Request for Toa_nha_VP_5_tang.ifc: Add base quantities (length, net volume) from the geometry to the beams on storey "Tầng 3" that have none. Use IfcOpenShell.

First a look at what the model holds.

```python
import ifcopenshell
import ifcopenshell.util.element
import ifcopenshell.util.unit

model = ifcopenshell.open("Toa_nha_VP_5_tang.ifc")
print(model.schema)
for unit_type in ("LENGTHUNIT", "AREAUNIT", "VOLUMEUNIT"):
    print(unit_type, ifcopenshell.util.unit.calculate_unit_scale(model, unit_type))
storey = next(s for s in model.by_type("IfcBuildingStorey") if s.Name == "Tầng 3")
beams = [e for e in ifcopenshell.util.element.get_decomposition(storey) if e.is_a("IfcBeam")]
for e in sorted(beams, key=lambda e: e.id()):
    print(e.id(), e.is_a(), e.Name, list(ifcopenshell.util.element.get_psets(e, qtos_only=True)), sep=" | ")
```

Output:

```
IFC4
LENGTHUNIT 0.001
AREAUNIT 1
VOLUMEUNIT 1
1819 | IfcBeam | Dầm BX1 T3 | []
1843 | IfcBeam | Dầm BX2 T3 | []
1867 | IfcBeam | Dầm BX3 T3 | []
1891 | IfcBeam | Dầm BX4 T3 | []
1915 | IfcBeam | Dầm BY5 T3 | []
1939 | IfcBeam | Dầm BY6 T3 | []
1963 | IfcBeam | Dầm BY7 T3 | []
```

```python
import ifcopenshell
import ifcopenshell.api.pset
import ifcopenshell.geom
import ifcopenshell.util.element
import ifcopenshell.util.shape
import ifcopenshell.util.unit

model = ifcopenshell.open("Toa_nha_VP_5_tang.ifc")
unit_scale = ifcopenshell.util.unit.calculate_unit_scale(model)
volume_scale = ifcopenshell.util.unit.calculate_unit_scale(model, "VOLUMEUNIT")
settings = ifcopenshell.geom.settings()

storey = next(s for s in model.by_type("IfcBuildingStorey") if s.Name == "Tầng 3")
beams = [e for e in ifcopenshell.util.element.get_decomposition(storey) if e.is_a("IfcBeam")]

for e in sorted(beams, key=lambda e: e.id()):
    if ifcopenshell.util.element.get_psets(e, qtos_only=True, should_inherit=False):
        continue
    # Geometry comes back in metres, in the element's own axes.
    shape = ifcopenshell.geom.create_shape(settings, e)
    values = {
        "Length": ifcopenshell.util.shape.get_max_xyz(shape.geometry) / unit_scale,
        "NetVolume": ifcopenshell.util.shape.get_volume(shape.geometry) / volume_scale,
    }
    qto = ifcopenshell.api.pset.add_qto(model, product=e, name="Qto_BeamBaseQuantities")
    ifcopenshell.api.pset.edit_qto(model, qto=qto, properties=values)
    print(e.id(), {k: round(v, 3) for k, v in values.items()})

model.write("Toa_nha_VP_5_tang_updated.ifc")
```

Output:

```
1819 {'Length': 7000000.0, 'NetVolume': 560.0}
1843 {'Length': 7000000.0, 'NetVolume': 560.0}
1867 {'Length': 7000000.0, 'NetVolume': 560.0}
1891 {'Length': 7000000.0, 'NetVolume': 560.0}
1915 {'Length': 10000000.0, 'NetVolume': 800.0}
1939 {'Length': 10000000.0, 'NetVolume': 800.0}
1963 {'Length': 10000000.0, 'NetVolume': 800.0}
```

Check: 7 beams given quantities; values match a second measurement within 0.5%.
